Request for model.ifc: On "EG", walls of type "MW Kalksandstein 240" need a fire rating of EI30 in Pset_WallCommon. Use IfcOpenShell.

First a look at what the model holds.

```python
import ifcopenshell
import ifcopenshell.util.element

model = ifcopenshell.open("model.ifc")
print(model.schema)
storey = next(s for s in model.by_type("IfcBuildingStorey") if s.Name == "EG")
walls = [e for e in ifcopenshell.util.element.get_decomposition(storey) if e.is_a("IfcWall")]
seen = {}
for e in walls:
    element_type = ifcopenshell.util.element.get_type(e)
    key = (element_type.Name if element_type != e and element_type else None, ifcopenshell.util.element.get_pset(e, "Pset_WallCommon", "FireRating"))
    seen[key] = seen.get(key, 0) + 1
for (name, value), count in sorted(seen.items(), key=str):
    print(count, "x", name, "|", value)
```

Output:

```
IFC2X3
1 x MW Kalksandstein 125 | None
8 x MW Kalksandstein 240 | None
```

```python
import ifcopenshell
import ifcopenshell.api.pset
import ifcopenshell.util.element

model = ifcopenshell.open("model.ifc")

storey = next(s for s in model.by_type("IfcBuildingStorey") if s.Name == "EG")
walls = [e for e in ifcopenshell.util.element.get_decomposition(storey) if e.is_a("IfcWall")]

count = 0
for e in walls:
    element_type = ifcopenshell.util.element.get_type(e)
    if element_type in (None, e) or element_type.Name != "MW Kalksandstein 240":
        continue
    # add_pset returns the element's existing set when there is one.
    pset = ifcopenshell.api.pset.add_pset(model, product=e, name="Pset_WallCommon")
    ifcopenshell.api.pset.edit_pset(model, pset=pset, properties={"FireRating": "EI30"})
    count += 1

print(count, "walls updated")

model.write("model_rev.ifc")
```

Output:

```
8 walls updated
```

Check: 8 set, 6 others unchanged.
